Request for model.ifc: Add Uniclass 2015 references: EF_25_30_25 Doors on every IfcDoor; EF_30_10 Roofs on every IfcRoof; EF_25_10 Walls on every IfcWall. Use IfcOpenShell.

First a look at what the model holds.

```python
import ifcopenshell

model = ifcopenshell.open("model.ifc")
print(model.schema)
print("classifications:", [c.Name for c in model.by_type("IfcClassification")])
for ifc_class in ("IfcDoor", "IfcRoof", "IfcStair", "IfcWall", "IfcWindow"):
    print(ifc_class, len(model.by_type(ifc_class)))
```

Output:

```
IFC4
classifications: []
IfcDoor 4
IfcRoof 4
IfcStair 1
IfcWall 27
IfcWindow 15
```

```python
import ifcopenshell
import ifcopenshell.api.classification

model = ifcopenshell.open("model.ifc")

system = ifcopenshell.api.classification.add_classification(model, classification="Uniclass 2015")

codes = {
    "IfcDoor": ("EF_25_30_25", "Doors"),
    "IfcRoof": ("EF_30_10", "Roofs"),
    "IfcWall": ("EF_25_10", "Walls"),
}
for ifc_class, (code, name) in codes.items():
    products = model.by_type(ifc_class)
    ifcopenshell.api.classification.add_reference(
        model, products=products, classification=system, identification=code, name=name
    )
    print(code, len(products))

model.write("model_edited.ifc")
```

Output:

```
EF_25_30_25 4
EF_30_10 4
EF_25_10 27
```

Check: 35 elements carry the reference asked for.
